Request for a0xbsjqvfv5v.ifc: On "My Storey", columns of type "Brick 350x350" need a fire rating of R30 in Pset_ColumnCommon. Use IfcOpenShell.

First a look at what the model holds.

```python
import ifcopenshell
import ifcopenshell.util.element

model = ifcopenshell.open("a0xbsjqvfv5v.ifc")
print(model.schema)
storey = next(s for s in model.by_type("IfcBuildingStorey") if s.Name == "My Storey")
columns = [e for e in ifcopenshell.util.element.get_decomposition(storey) if e.is_a("IfcColumn")]
seen = {}
for e in columns:
    element_type = ifcopenshell.util.element.get_type(e)
    key = (element_type.Name if element_type != e and element_type else None, ifcopenshell.util.element.get_pset(e, "Pset_ColumnCommon", "FireRating"))
    seen[key] = seen.get(key, 0) + 1
for (name, value), count in sorted(seen.items(), key=str):
    print(count, "x", name, "|", value)
```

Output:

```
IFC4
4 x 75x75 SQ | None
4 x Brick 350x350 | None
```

```python
import ifcopenshell
import ifcopenshell.api.pset
import ifcopenshell.util.element

model = ifcopenshell.open("a0xbsjqvfv5v.ifc")

storey = next(s for s in model.by_type("IfcBuildingStorey") if s.Name == "My Storey")
columns = [e for e in ifcopenshell.util.element.get_decomposition(storey) if e.is_a("IfcColumn")]

count = 0
for e in columns:
    element_type = ifcopenshell.util.element.get_type(e)
    if element_type in (None, e) or element_type.Name != "Brick 350x350":
        continue
    # add_pset returns the element's existing set when there is one.
    pset = ifcopenshell.api.pset.add_pset(model, product=e, name="Pset_ColumnCommon")
    ifcopenshell.api.pset.edit_pset(model, pset=pset, properties={"FireRating": "R30"})
    count += 1

print(count, "columns updated")

model.write("a0xbsjqvfv5v_rev.ifc")
```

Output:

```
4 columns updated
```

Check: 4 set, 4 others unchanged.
